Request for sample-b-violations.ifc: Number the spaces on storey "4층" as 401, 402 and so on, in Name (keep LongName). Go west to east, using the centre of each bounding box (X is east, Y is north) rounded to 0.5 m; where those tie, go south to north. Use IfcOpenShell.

First a look at what the model holds.

```python
import ifcopenshell
import ifcopenshell.util.element
import ifcopenshell.util.placement

model = ifcopenshell.open("sample-b-violations.ifc")
print(model.schema)
storey = next(s for s in model.by_type("IfcBuildingStorey") if s.Name == "4층")
spaces = [e for e in ifcopenshell.util.element.get_decomposition(storey) if e.is_a("IfcSpace")]
for e in sorted(spaces, key=lambda e: e.id()):
    origin = ifcopenshell.util.placement.get_local_placement(e.ObjectPlacement)[:3, 3]
    print(e.id(), e.Name, e.LongName, origin.round(2) + 0.0, sep=" | ")
```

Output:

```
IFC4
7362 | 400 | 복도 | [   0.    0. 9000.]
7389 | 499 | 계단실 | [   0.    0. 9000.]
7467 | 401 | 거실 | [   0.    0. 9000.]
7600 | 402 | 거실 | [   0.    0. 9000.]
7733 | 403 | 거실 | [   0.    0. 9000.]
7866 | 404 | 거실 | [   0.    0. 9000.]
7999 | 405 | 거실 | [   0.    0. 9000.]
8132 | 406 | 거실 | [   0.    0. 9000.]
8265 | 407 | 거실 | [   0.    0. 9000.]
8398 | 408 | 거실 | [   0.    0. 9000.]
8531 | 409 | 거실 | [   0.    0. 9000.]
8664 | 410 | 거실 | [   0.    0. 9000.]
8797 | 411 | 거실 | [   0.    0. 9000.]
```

```python
import ifcopenshell
import ifcopenshell.geom
import ifcopenshell.util.element
import ifcopenshell.util.shape

model = ifcopenshell.open("sample-b-violations.ifc")
settings = ifcopenshell.geom.settings()
settings.set("use-world-coords", True)


def centre(element):
    shape = ifcopenshell.geom.create_shape(settings, element)
    return ifcopenshell.util.shape.get_bbox_centroid(shape.geometry)


storey = next(s for s in model.by_type("IfcBuildingStorey") if s.Name == "4층")
spaces = [e for e in ifcopenshell.util.element.get_decomposition(storey) if e.is_a("IfcSpace")]

# Insertion points can sit at a corner or the storey origin, so sort by the geometry (in metres).
centres = {e: centre(e) for e in spaces}
spaces.sort(key=lambda e: (round(centres[e][0] / 0.5), centres[e][1]))

for i, e in enumerate(spaces, start=1):
    number = f"4{i:02d}"
    e.Name = number
    print(e.id(), number)

model.write("sample-b-violations_edited.ifc")
```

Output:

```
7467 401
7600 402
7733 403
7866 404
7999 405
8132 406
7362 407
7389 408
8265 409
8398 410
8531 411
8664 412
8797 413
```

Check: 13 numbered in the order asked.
